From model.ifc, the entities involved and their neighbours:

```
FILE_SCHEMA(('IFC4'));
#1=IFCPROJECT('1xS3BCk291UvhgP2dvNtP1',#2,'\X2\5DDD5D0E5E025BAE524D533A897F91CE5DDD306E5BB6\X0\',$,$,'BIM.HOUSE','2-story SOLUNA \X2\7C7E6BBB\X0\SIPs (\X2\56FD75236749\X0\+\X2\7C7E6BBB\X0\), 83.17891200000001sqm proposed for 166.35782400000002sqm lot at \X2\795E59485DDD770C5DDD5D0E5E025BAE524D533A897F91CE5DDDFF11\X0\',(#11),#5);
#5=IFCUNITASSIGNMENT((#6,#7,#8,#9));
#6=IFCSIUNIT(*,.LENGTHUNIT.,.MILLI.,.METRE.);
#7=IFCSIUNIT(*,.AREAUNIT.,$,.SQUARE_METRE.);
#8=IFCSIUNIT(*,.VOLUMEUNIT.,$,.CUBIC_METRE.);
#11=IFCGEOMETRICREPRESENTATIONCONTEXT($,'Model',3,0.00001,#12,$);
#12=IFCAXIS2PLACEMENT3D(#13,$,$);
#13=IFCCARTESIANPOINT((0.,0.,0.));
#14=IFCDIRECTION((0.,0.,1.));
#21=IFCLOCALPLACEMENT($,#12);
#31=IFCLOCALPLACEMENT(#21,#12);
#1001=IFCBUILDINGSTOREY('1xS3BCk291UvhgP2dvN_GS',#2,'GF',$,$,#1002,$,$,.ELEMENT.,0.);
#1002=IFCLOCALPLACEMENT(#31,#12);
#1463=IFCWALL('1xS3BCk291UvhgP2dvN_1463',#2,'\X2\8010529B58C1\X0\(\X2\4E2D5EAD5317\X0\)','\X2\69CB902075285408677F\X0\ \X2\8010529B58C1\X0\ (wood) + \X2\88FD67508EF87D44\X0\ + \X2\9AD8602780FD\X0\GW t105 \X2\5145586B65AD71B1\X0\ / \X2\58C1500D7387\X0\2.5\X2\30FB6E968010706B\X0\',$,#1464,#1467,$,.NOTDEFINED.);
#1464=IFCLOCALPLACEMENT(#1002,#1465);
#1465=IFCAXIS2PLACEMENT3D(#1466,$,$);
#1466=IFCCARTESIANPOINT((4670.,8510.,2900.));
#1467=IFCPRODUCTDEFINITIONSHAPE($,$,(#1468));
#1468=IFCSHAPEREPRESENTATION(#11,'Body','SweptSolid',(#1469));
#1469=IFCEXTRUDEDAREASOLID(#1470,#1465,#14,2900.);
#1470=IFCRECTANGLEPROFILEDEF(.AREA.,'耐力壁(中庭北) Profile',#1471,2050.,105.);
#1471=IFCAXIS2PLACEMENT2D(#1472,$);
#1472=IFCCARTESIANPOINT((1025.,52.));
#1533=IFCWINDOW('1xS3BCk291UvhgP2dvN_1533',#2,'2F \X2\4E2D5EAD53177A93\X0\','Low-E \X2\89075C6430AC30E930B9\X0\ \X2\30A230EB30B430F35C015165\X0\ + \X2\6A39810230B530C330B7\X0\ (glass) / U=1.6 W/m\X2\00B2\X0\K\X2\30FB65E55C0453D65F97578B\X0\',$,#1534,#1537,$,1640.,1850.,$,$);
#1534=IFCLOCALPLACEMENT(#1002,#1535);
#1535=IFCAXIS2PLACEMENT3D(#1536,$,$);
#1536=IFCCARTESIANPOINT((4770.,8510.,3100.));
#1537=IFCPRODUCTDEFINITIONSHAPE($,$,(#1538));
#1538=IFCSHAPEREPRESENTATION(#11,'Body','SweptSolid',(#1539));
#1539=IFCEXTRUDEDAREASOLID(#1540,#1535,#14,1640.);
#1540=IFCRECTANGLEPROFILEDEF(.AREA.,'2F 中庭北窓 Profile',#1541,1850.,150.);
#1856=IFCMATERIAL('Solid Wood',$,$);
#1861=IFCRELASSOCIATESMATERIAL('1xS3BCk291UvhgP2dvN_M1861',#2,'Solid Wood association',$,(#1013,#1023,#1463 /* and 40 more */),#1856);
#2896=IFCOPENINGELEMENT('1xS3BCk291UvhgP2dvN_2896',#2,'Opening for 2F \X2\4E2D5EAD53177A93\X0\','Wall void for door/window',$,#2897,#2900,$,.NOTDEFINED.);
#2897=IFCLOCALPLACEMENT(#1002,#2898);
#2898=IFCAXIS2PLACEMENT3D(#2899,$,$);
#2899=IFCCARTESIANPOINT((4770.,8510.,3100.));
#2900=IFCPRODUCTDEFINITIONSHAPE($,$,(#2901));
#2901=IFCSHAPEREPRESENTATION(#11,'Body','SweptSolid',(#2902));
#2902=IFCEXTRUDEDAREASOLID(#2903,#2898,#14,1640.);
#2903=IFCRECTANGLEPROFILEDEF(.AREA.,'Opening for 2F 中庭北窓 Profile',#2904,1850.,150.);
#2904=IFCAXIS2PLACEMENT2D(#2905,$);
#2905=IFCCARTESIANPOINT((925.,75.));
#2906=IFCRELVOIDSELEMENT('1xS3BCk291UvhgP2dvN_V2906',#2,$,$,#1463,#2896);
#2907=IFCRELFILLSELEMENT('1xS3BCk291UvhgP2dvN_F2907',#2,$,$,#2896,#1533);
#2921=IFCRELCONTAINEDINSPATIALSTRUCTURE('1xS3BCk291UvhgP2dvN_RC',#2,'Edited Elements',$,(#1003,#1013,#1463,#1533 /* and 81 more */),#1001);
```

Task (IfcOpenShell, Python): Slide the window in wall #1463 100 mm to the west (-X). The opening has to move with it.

```python
import ifcopenshell
import ifcopenshell.api.geometry
import ifcopenshell.util.placement
import ifcopenshell.util.unit

model = ifcopenshell.open("model.ifc")
unit_scale = ifcopenshell.util.unit.calculate_unit_scale(model)

window = model.by_guid("1xS3BCk291UvhgP2dvN_1533")
opening = window.FillsVoids[0].RelatingOpeningElement
wall = opening.VoidsElements[0].RelatingBuildingElement

wall_matrix = ifcopenshell.util.placement.get_local_placement(wall.ObjectPlacement)
shift = wall_matrix[:3, 0] * -0.1 / unit_scale
before = ifcopenshell.util.placement.get_local_placement(window.ObjectPlacement)[:3, 3].copy()

# The window is not placed relative to its opening, so move both.
for product in (opening, window):
    matrix = ifcopenshell.util.placement.get_local_placement(product.ObjectPlacement)
    matrix[:3, 3] += shift
    ifcopenshell.api.geometry.edit_object_placement(model, product=product, matrix=matrix, is_si=False)

after = ifcopenshell.util.placement.get_local_placement(window.ObjectPlacement)[:3, 3]
print("window moved by", (after - before).round(3) + 0.0)

model.write("model_rev.ifc")
```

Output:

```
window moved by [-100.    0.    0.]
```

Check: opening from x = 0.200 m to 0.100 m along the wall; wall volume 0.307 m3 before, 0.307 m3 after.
